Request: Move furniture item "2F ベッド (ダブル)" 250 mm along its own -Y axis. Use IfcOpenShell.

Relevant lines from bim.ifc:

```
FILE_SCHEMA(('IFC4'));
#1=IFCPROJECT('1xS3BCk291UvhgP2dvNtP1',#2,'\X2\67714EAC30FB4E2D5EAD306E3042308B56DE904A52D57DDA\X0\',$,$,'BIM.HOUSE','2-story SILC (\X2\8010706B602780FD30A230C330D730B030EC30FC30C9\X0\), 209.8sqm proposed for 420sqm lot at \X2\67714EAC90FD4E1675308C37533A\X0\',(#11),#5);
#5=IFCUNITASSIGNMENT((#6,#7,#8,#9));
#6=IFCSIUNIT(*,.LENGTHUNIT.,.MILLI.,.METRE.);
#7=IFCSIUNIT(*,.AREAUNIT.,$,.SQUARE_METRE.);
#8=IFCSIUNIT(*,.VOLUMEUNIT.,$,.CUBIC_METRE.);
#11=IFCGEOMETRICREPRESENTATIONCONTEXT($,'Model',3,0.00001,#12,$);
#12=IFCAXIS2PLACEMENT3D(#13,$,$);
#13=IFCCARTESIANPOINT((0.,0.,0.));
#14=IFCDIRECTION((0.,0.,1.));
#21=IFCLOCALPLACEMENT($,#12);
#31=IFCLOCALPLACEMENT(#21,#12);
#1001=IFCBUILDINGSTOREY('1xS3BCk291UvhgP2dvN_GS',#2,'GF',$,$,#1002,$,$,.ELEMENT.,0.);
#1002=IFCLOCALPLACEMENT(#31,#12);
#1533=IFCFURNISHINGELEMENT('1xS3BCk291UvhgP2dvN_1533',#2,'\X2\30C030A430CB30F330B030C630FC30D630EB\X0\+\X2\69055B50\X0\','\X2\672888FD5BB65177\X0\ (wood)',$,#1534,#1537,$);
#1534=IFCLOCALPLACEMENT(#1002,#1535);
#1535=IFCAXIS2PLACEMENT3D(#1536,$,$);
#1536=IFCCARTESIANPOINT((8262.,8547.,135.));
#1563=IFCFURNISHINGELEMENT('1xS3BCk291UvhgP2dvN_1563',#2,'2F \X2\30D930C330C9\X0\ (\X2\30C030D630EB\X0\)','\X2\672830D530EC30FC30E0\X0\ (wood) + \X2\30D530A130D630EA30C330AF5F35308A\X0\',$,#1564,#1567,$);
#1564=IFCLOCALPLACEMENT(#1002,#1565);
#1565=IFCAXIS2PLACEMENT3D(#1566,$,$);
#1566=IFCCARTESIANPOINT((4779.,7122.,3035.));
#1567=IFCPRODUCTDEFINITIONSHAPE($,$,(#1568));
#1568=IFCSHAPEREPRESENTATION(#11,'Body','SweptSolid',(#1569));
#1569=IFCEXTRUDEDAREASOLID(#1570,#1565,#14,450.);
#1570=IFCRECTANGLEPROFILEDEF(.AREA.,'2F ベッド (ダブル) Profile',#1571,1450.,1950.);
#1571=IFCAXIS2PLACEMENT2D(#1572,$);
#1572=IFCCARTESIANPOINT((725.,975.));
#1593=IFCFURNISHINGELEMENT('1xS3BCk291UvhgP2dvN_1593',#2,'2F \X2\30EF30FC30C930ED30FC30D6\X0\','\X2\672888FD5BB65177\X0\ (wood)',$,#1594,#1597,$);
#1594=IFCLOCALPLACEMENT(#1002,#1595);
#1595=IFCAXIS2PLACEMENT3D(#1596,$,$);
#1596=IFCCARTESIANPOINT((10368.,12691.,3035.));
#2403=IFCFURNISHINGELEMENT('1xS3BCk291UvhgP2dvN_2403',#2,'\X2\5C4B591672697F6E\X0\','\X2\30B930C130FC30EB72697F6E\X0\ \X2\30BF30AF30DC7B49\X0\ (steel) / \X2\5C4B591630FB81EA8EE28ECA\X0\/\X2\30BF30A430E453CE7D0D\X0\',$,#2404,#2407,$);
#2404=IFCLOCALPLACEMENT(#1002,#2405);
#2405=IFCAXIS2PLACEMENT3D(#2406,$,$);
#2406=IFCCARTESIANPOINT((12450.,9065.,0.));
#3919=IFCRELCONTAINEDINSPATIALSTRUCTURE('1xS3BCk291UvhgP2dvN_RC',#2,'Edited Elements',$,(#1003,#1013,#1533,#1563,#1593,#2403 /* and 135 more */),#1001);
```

```python
import ifcopenshell
import ifcopenshell.api.geometry
import ifcopenshell.util.placement
import ifcopenshell.util.unit

model = ifcopenshell.open("bim.ifc")
unit_scale = ifcopenshell.util.unit.calculate_unit_scale(model)

item = model.by_guid("1xS3BCk291UvhgP2dvN_1563")
matrix = ifcopenshell.util.placement.get_local_placement(item.ObjectPlacement)
matrix[:3, 3] -= matrix[:3, 1] * 0.25 / unit_scale
ifcopenshell.api.geometry.edit_object_placement(model, product=item, matrix=matrix, is_si=False)

print(ifcopenshell.util.placement.get_local_placement(item.ObjectPlacement).round(3) + 0.0)

model.write("bim_v2.ifc")
```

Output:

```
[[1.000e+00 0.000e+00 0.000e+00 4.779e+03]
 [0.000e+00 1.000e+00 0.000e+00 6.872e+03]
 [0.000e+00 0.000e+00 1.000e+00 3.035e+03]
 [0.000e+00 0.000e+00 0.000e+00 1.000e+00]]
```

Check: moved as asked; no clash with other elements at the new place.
